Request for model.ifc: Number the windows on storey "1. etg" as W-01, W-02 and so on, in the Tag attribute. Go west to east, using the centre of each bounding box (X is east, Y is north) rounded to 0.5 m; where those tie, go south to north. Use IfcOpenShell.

First a look at what the model holds.

```python
import ifcopenshell
import ifcopenshell.util.element
import ifcopenshell.util.placement

model = ifcopenshell.open("model.ifc")
print(model.schema)
storey = next(s for s in model.by_type("IfcBuildingStorey") if s.Name == "1. etg")
windows = [e for e in ifcopenshell.util.element.get_decomposition(storey) if e.is_a("IfcWindow")]
for e in sorted(windows, key=lambda e: e.id()):
    origin = ifcopenshell.util.placement.get_local_placement(e.ObjectPlacement)[:3, 3]
    print(e.id(), e.Tag, e.Name, origin.round(2) + 0.0, sep=" | ")
```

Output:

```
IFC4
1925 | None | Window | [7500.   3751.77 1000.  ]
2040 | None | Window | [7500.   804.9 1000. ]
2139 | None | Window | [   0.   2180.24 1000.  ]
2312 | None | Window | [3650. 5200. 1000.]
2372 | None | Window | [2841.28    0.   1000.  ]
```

```python
import ifcopenshell
import ifcopenshell.geom
import ifcopenshell.util.element
import ifcopenshell.util.shape

model = ifcopenshell.open("model.ifc")
settings = ifcopenshell.geom.settings()
settings.set("use-world-coords", True)


def centre(element):
    shape = ifcopenshell.geom.create_shape(settings, element)
    return ifcopenshell.util.shape.get_bbox_centroid(shape.geometry)


storey = next(s for s in model.by_type("IfcBuildingStorey") if s.Name == "1. etg")
windows = [e for e in ifcopenshell.util.element.get_decomposition(storey) if e.is_a("IfcWindow")]

# Insertion points can sit at a corner or the storey origin, so sort by the geometry (in metres).
centres = {e: centre(e) for e in windows}
windows.sort(key=lambda e: (round(centres[e][0] / 0.5), centres[e][1]))

for i, e in enumerate(windows, start=1):
    number = f"W-{i:02d}"
    e.Tag = number
    print(e.id(), number)

model.write("model_rev.ifc")
```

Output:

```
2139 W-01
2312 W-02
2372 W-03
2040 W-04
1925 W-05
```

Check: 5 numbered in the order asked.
